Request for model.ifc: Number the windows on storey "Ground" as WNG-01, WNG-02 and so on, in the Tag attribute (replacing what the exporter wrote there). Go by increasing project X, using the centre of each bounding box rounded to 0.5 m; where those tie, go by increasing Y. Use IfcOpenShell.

First a look at what the model holds.

```python
import ifcopenshell
import ifcopenshell.util.element
import ifcopenshell.util.placement

model = ifcopenshell.open("model.ifc")
print(model.schema)
storey = next(s for s in model.by_type("IfcBuildingStorey") if s.Name == "Ground")
windows = [e for e in ifcopenshell.util.element.get_decomposition(storey) if e.is_a("IfcWindow")]
for e in sorted(windows, key=lambda e: e.id()):
    origin = ifcopenshell.util.placement.get_local_placement(e.ObjectPlacement)[:3, 3]
    print(e.id(), e.Tag, e.Name, origin.round(2) + 0.0, sep=" | ")
```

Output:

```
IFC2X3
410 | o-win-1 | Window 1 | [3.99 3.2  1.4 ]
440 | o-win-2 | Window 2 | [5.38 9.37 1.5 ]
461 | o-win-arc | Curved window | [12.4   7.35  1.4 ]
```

```python
import ifcopenshell
import ifcopenshell.geom
import ifcopenshell.util.element
import ifcopenshell.util.shape

model = ifcopenshell.open("model.ifc")
settings = ifcopenshell.geom.settings()
settings.set("use-world-coords", True)


def centre(element):
    shape = ifcopenshell.geom.create_shape(settings, element)
    return ifcopenshell.util.shape.get_bbox_centroid(shape.geometry)


storey = next(s for s in model.by_type("IfcBuildingStorey") if s.Name == "Ground")
windows = [e for e in ifcopenshell.util.element.get_decomposition(storey) if e.is_a("IfcWindow")]

# Insertion points can sit at a corner or the storey origin, so sort by the geometry (in metres).
centres = {e: centre(e) for e in windows}
windows.sort(key=lambda e: (round(centres[e][0] / 0.5), centres[e][1]))

for i, e in enumerate(windows, start=1):
    number = f"WNG-{i:02d}"
    e.Tag = number
    print(e.id(), number)

model.write("model_edited.ifc")
```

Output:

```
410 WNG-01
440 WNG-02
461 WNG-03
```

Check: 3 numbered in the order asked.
